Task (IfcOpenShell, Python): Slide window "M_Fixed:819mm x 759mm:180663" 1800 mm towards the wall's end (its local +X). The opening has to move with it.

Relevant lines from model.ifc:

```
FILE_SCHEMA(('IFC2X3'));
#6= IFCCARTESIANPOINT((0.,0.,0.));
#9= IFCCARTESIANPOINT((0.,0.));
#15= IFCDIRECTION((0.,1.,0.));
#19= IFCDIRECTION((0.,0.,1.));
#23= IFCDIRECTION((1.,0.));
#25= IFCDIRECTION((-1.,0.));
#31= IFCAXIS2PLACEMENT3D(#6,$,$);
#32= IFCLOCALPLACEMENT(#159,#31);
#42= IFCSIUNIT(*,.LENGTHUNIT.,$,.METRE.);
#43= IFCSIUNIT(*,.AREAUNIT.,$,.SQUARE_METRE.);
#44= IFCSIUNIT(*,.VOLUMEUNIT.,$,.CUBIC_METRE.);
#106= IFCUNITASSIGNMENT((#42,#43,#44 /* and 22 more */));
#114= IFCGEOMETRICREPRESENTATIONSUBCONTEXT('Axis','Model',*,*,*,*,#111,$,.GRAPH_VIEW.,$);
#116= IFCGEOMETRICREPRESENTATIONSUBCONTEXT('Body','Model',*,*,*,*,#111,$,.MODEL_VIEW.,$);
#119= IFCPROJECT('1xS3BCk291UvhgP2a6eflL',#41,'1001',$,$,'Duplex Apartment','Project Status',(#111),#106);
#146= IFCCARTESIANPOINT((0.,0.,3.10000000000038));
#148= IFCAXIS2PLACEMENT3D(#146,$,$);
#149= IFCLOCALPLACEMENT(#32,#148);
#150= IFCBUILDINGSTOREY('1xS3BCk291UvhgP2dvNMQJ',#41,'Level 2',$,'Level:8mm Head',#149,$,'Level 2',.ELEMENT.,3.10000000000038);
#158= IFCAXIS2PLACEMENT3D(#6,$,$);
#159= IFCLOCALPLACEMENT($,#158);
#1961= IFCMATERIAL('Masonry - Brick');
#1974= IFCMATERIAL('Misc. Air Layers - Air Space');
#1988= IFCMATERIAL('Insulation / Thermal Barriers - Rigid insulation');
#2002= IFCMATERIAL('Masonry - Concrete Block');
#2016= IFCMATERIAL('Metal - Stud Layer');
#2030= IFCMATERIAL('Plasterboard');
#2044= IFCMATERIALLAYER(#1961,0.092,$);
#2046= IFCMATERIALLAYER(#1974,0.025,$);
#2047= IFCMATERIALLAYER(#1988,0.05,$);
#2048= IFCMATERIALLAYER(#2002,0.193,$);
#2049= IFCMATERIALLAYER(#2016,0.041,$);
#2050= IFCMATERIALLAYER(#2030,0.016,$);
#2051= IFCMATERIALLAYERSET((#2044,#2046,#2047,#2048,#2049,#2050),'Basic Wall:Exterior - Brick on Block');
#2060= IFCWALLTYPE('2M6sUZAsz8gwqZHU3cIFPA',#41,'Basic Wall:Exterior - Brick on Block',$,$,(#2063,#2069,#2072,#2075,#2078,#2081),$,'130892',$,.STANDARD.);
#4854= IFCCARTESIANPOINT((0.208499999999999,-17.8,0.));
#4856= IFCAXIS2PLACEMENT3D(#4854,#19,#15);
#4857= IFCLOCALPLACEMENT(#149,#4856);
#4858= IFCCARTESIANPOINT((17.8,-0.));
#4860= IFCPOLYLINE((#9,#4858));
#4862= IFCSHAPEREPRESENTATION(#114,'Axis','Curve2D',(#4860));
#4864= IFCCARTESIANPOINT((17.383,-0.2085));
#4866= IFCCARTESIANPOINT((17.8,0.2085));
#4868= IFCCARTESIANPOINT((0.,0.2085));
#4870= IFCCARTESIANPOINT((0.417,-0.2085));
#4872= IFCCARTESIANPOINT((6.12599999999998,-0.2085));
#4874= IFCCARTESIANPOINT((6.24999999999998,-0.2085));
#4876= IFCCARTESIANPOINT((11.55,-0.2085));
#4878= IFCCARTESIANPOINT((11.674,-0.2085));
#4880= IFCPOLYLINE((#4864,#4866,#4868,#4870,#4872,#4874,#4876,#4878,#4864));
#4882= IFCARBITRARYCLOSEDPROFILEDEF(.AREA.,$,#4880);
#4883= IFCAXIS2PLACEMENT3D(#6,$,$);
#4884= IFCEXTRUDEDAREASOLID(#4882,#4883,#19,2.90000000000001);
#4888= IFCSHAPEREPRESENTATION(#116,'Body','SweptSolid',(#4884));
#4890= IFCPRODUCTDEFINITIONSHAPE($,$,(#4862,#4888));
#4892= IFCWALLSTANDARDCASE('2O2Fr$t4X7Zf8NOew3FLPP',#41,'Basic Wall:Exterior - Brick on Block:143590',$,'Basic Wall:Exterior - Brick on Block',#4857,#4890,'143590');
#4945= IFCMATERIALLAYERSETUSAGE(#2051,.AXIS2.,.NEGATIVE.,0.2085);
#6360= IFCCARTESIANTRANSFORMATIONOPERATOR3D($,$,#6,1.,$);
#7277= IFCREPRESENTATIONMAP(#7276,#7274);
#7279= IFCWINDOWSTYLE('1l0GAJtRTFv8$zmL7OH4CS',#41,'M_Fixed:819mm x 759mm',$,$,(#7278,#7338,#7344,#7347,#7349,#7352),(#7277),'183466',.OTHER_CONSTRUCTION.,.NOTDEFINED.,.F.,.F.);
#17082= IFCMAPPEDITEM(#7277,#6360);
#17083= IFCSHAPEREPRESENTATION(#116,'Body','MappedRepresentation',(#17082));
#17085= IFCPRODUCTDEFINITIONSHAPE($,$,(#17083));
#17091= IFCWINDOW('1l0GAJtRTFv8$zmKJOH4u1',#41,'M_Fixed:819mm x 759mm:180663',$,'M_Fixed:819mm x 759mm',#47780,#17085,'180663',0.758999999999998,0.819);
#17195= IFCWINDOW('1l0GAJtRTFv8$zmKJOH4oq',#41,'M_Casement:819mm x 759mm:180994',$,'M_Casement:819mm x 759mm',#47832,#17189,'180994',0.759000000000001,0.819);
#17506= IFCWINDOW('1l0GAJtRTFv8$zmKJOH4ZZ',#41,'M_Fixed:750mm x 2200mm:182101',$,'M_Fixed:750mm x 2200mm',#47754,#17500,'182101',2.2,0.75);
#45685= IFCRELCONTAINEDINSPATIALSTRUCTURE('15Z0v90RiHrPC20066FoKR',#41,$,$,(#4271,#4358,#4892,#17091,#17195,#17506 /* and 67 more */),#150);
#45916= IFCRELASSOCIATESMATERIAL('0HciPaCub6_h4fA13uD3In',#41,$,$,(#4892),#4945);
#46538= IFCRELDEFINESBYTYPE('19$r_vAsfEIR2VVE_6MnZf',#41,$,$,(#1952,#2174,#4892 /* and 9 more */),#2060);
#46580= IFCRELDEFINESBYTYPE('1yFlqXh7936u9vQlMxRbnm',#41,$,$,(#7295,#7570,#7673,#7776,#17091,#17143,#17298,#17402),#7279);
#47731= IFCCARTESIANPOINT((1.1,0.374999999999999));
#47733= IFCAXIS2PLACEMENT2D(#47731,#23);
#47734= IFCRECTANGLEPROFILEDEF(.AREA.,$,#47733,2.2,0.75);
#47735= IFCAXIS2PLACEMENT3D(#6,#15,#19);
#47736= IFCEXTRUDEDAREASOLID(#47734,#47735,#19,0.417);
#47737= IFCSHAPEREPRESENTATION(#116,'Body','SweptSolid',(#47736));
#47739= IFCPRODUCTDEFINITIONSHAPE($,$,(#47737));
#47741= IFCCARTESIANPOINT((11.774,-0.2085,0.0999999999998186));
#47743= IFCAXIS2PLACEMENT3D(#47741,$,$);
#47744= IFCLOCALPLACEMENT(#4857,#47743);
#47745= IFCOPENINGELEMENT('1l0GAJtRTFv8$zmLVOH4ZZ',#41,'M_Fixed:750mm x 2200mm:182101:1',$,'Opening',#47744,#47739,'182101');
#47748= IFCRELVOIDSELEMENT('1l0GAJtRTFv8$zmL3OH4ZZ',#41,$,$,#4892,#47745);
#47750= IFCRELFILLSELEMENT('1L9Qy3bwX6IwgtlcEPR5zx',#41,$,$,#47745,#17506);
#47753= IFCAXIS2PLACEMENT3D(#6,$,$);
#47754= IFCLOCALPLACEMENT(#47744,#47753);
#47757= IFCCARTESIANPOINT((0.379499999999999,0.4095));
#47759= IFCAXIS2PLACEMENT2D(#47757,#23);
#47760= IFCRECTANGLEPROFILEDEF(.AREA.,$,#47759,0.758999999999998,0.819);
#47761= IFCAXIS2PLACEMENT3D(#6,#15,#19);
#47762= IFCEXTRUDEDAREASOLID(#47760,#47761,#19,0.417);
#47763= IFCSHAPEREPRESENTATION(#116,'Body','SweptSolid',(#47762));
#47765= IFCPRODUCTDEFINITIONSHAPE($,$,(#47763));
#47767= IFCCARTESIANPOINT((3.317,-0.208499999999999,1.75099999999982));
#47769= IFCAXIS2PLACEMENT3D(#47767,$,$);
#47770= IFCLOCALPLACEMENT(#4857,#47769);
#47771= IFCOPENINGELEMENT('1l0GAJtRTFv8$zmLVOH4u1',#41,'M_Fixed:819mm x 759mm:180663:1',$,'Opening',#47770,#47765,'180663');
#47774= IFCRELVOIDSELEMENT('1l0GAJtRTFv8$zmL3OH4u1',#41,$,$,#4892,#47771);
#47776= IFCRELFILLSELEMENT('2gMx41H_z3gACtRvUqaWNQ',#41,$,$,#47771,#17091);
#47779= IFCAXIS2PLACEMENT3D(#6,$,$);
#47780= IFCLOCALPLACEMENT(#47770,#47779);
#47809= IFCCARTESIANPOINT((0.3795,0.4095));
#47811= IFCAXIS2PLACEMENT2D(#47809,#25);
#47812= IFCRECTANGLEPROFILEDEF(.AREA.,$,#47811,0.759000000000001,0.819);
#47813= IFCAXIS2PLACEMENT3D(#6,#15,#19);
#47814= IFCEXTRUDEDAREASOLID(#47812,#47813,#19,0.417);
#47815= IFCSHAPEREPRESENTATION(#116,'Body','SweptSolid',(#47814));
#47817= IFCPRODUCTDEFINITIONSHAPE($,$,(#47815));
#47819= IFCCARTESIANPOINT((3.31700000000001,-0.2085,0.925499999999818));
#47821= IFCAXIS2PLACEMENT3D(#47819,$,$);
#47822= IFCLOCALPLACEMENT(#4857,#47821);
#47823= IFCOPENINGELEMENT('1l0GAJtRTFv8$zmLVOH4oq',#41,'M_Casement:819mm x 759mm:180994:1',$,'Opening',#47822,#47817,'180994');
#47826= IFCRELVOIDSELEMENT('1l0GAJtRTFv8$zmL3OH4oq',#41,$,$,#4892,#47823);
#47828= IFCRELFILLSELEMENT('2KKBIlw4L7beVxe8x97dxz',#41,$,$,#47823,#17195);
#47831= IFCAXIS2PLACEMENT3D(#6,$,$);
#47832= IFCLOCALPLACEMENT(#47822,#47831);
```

```python
import ifcopenshell
import ifcopenshell.api.geometry
import ifcopenshell.util.placement

model = ifcopenshell.open("model.ifc")

window = model.by_guid("1l0GAJtRTFv8$zmKJOH4u1")
opening = window.FillsVoids[0].RelatingOpeningElement
wall = opening.VoidsElements[0].RelatingBuildingElement

wall_matrix = ifcopenshell.util.placement.get_local_placement(wall.ObjectPlacement)
shift = wall_matrix[:3, 0] * 1.8
before = ifcopenshell.util.placement.get_local_placement(window.ObjectPlacement)[:3, 3].copy()

# The window is placed relative to its opening, so it follows when the opening moves.
matrix = ifcopenshell.util.placement.get_local_placement(opening.ObjectPlacement)
matrix[:3, 3] += shift
ifcopenshell.api.geometry.edit_object_placement(
    model, product=opening, matrix=matrix, is_si=False, should_transform_children=True
)

after = ifcopenshell.util.placement.get_local_placement(window.ObjectPlacement)[:3, 3]
print("window moved by", (after - before).round(3) + 0.0)

model.write("model_rev.ifc")
```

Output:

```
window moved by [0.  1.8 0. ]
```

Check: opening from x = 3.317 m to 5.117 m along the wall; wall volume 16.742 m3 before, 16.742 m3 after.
